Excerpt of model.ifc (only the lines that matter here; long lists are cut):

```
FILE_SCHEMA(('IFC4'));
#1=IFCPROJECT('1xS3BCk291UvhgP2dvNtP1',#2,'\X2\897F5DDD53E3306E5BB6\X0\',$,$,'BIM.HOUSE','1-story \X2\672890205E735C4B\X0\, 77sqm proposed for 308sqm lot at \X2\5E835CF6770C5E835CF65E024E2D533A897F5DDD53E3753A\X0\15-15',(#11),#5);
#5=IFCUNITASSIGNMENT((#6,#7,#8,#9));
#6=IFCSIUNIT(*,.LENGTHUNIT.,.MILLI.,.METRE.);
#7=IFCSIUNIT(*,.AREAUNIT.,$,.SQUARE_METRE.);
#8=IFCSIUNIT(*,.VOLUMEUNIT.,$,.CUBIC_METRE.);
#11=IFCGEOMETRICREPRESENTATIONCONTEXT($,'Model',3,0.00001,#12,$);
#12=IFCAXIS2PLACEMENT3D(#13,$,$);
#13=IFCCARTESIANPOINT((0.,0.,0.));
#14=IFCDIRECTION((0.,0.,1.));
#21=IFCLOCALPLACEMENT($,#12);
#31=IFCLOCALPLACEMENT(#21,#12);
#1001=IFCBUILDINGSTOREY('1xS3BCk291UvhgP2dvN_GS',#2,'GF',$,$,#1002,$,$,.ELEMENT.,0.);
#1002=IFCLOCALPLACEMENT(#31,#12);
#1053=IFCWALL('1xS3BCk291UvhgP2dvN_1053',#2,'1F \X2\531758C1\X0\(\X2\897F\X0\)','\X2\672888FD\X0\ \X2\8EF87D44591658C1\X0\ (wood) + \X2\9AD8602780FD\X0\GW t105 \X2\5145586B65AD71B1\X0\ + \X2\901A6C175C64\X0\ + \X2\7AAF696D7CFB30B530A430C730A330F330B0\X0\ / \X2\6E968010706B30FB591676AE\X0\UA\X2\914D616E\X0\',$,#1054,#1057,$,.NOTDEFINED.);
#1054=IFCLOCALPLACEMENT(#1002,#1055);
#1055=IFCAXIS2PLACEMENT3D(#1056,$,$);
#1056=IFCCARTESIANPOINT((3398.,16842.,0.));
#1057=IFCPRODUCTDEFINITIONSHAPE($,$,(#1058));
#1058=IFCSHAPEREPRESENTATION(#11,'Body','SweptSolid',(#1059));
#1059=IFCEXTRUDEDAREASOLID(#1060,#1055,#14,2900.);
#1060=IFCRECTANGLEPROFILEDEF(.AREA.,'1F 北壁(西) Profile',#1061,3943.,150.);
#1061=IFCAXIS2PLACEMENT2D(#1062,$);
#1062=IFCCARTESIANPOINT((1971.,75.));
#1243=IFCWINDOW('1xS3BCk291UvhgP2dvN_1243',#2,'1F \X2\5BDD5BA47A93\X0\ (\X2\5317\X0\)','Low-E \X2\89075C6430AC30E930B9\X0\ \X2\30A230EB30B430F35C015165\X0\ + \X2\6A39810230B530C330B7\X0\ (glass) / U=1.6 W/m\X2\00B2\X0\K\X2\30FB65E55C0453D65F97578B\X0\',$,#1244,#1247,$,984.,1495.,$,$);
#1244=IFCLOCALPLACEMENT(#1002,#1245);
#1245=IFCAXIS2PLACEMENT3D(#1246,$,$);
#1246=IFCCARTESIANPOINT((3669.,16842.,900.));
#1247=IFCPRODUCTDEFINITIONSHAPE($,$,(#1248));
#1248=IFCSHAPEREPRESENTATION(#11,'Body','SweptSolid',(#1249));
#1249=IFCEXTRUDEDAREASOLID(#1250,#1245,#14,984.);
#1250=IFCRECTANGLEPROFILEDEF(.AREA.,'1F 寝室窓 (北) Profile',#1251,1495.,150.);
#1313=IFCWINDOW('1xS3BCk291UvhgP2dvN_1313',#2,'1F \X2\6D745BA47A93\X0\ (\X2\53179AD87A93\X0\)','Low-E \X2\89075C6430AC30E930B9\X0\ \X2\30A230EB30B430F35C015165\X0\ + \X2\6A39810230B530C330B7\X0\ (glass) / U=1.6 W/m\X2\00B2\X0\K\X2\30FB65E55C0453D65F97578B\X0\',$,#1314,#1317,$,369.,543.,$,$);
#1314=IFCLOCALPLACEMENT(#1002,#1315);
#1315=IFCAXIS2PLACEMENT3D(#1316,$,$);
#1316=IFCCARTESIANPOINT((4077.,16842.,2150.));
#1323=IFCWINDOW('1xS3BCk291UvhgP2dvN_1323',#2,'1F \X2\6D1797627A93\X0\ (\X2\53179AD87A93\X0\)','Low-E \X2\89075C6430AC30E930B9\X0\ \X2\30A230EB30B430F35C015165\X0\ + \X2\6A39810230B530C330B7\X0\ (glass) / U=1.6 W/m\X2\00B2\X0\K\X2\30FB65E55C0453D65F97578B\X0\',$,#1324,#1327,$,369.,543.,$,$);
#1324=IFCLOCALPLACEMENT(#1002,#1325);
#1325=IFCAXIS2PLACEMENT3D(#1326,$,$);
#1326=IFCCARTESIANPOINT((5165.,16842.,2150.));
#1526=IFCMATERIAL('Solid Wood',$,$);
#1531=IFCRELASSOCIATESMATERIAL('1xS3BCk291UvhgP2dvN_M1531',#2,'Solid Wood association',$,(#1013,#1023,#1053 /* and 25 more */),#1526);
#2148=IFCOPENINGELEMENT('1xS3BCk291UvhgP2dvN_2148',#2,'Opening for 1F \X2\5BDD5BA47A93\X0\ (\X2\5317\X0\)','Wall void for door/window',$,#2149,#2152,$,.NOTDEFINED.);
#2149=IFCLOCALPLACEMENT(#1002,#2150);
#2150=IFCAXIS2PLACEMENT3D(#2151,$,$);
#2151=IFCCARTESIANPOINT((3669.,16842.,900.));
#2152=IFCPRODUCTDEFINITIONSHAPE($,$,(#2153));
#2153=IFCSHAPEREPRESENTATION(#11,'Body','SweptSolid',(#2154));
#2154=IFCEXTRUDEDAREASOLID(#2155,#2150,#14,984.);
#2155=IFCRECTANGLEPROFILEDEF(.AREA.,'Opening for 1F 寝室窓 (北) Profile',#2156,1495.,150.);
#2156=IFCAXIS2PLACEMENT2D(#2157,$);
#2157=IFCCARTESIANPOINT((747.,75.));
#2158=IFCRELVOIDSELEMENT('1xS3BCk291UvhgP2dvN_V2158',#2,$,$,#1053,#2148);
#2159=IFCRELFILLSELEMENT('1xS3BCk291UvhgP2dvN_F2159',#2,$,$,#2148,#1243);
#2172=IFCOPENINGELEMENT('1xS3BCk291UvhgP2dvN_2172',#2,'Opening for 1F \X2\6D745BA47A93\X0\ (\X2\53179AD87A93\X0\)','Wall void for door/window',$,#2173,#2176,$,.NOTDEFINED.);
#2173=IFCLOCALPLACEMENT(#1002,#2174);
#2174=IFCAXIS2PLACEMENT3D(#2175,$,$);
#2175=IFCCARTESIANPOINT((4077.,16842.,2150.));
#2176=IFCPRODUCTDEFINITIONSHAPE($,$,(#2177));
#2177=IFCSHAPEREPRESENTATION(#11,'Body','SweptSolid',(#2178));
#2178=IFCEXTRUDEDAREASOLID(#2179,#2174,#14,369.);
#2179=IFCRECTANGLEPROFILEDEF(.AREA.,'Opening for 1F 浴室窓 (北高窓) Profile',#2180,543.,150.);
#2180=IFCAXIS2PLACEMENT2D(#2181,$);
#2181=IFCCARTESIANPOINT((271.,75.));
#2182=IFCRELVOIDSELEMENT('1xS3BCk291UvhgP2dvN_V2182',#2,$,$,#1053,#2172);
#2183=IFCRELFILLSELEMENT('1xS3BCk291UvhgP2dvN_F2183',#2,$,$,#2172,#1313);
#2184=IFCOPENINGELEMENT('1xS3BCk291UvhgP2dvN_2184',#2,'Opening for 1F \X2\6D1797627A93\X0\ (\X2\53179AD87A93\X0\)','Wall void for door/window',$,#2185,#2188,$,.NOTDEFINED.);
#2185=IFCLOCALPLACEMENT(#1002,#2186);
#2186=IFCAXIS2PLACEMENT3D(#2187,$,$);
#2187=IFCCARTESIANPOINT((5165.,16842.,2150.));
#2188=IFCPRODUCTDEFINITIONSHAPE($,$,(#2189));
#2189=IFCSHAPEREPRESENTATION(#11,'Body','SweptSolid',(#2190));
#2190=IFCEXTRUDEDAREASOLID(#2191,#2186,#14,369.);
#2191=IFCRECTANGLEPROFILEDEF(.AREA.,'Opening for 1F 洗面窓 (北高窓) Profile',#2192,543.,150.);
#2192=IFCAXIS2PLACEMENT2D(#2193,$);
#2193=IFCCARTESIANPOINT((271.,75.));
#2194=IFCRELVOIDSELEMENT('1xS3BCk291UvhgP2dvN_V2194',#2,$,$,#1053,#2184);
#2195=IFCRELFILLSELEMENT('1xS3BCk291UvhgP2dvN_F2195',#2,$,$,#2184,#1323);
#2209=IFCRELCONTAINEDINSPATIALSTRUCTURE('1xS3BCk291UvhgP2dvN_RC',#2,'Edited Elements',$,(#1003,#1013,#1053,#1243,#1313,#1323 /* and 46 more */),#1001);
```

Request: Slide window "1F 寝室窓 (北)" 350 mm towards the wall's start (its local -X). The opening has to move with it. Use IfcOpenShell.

```python
import ifcopenshell
import ifcopenshell.api.geometry
import ifcopenshell.util.placement
import ifcopenshell.util.unit

model = ifcopenshell.open("model.ifc")
unit_scale = ifcopenshell.util.unit.calculate_unit_scale(model)

window = model.by_guid("1xS3BCk291UvhgP2dvN_1243")
opening = window.FillsVoids[0].RelatingOpeningElement
wall = opening.VoidsElements[0].RelatingBuildingElement

wall_matrix = ifcopenshell.util.placement.get_local_placement(wall.ObjectPlacement)
shift = wall_matrix[:3, 0] * -0.35 / unit_scale
before = ifcopenshell.util.placement.get_local_placement(window.ObjectPlacement)[:3, 3].copy()

# The window is not placed relative to its opening, so move both.
for product in (opening, window):
    matrix = ifcopenshell.util.placement.get_local_placement(product.ObjectPlacement)
    matrix[:3, 3] += shift
    ifcopenshell.api.geometry.edit_object_placement(model, product=product, matrix=matrix, is_si=False)

after = ifcopenshell.util.placement.get_local_placement(window.ObjectPlacement)[:3, 3]
print("window moved by", (after - before).round(3) + 0.0)

model.write("model_v2.ifc")
```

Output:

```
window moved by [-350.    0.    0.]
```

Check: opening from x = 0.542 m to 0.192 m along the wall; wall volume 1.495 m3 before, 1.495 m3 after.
